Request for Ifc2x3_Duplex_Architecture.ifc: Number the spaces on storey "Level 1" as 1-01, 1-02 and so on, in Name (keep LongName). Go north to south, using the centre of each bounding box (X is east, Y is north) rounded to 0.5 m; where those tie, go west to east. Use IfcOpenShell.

First a look at what the model holds.

```python
import ifcopenshell
import ifcopenshell.util.element
import ifcopenshell.util.placement

model = ifcopenshell.open("Ifc2x3_Duplex_Architecture.ifc")
print(model.schema)
storey = next(s for s in model.by_type("IfcBuildingStorey") if s.Name == "Level 1")
spaces = [e for e in ifcopenshell.util.element.get_decomposition(storey) if e.is_a("IfcSpace")]
for e in sorted(spaces, key=lambda e: e.id()):
    origin = ifcopenshell.util.placement.get_local_placement(e.ObjectPlacement)[:3, 3]
    print(e.id(), e.Name, e.LongName, origin.round(2) + 0.0, sep=" | ")
```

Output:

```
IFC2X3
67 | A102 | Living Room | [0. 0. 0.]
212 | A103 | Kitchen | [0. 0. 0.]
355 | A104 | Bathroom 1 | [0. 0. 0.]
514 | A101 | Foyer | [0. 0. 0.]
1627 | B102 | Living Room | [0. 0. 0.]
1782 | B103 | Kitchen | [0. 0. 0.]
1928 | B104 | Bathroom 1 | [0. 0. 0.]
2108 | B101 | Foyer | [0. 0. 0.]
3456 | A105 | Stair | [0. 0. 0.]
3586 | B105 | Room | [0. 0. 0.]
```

```python
import ifcopenshell
import ifcopenshell.geom
import ifcopenshell.util.element
import ifcopenshell.util.shape

model = ifcopenshell.open("Ifc2x3_Duplex_Architecture.ifc")
settings = ifcopenshell.geom.settings()
settings.set("use-world-coords", True)


def centre(element):
    shape = ifcopenshell.geom.create_shape(settings, element)
    return ifcopenshell.util.shape.get_bbox_centroid(shape.geometry)


storey = next(s for s in model.by_type("IfcBuildingStorey") if s.Name == "Level 1")
spaces = [e for e in ifcopenshell.util.element.get_decomposition(storey) if e.is_a("IfcSpace")]

# Insertion points can sit at a corner or the storey origin, so sort by the geometry (in metres).
centres = {e: centre(e) for e in spaces}
spaces.sort(key=lambda e: (-round(centres[e][1] / 0.5), centres[e][0]))

for i, e in enumerate(spaces, start=1):
    number = f"1-{i:02d}"
    e.Name = number
    print(e.id(), number)

model.write("Ifc2x3_Duplex_Architecture-out.ifc")
```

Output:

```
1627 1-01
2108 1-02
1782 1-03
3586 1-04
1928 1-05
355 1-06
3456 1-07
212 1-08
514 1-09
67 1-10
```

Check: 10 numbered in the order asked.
